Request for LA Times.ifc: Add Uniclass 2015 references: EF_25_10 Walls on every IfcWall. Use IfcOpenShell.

First a look at what the model holds.

```python
import ifcopenshell

model = ifcopenshell.open("LA Times.ifc")
print(model.schema)
print("classifications:", [c.Name for c in model.by_type("IfcClassification")])
for ifc_class in ("IfcDoor", "IfcRoof", "IfcStair", "IfcWall", "IfcWindow"):
    print(ifc_class, len(model.by_type(ifc_class)))
```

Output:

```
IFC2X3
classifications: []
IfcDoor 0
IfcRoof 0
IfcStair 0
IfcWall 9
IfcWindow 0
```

```python
import ifcopenshell
import ifcopenshell.api.classification

model = ifcopenshell.open("LA Times.ifc")

# IFC2X3 requires Source and Edition and has no link from the project to the system.
system = model.create_entity("IfcClassification", Source="NBS", Edition="2015", Name="Uniclass 2015")

codes = {
    "IfcWall": ("EF_25_10", "Walls"),
}
for ifc_class, (code, name) in codes.items():
    products = model.by_type(ifc_class)
    ifcopenshell.api.classification.add_reference(
        model, products=products, classification=system, identification=code, name=name
    )
    print(code, len(products))

model.write("LA Times_updated.ifc")
```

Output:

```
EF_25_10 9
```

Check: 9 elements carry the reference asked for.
